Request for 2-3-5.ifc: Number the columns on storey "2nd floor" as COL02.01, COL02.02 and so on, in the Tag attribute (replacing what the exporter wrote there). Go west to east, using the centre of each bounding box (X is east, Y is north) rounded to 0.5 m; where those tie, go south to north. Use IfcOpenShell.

First a look at what the model holds.

```python
import ifcopenshell
import ifcopenshell.util.element
import ifcopenshell.util.placement

model = ifcopenshell.open("2-3-5.ifc")
print(model.schema)
storey = next(s for s in model.by_type("IfcBuildingStorey") if s.Name == "2nd floor")
columns = [e for e in ifcopenshell.util.element.get_decomposition(storey) if e.is_a("IfcColumn")]
for e in sorted(columns, key=lambda e: e.id()):
    origin = ifcopenshell.util.placement.get_local_placement(e.ObjectPlacement)[:3, 3]
    print(e.id(), e.Tag, e.Name, origin.round(2) + 0.0, sep=" | ")
```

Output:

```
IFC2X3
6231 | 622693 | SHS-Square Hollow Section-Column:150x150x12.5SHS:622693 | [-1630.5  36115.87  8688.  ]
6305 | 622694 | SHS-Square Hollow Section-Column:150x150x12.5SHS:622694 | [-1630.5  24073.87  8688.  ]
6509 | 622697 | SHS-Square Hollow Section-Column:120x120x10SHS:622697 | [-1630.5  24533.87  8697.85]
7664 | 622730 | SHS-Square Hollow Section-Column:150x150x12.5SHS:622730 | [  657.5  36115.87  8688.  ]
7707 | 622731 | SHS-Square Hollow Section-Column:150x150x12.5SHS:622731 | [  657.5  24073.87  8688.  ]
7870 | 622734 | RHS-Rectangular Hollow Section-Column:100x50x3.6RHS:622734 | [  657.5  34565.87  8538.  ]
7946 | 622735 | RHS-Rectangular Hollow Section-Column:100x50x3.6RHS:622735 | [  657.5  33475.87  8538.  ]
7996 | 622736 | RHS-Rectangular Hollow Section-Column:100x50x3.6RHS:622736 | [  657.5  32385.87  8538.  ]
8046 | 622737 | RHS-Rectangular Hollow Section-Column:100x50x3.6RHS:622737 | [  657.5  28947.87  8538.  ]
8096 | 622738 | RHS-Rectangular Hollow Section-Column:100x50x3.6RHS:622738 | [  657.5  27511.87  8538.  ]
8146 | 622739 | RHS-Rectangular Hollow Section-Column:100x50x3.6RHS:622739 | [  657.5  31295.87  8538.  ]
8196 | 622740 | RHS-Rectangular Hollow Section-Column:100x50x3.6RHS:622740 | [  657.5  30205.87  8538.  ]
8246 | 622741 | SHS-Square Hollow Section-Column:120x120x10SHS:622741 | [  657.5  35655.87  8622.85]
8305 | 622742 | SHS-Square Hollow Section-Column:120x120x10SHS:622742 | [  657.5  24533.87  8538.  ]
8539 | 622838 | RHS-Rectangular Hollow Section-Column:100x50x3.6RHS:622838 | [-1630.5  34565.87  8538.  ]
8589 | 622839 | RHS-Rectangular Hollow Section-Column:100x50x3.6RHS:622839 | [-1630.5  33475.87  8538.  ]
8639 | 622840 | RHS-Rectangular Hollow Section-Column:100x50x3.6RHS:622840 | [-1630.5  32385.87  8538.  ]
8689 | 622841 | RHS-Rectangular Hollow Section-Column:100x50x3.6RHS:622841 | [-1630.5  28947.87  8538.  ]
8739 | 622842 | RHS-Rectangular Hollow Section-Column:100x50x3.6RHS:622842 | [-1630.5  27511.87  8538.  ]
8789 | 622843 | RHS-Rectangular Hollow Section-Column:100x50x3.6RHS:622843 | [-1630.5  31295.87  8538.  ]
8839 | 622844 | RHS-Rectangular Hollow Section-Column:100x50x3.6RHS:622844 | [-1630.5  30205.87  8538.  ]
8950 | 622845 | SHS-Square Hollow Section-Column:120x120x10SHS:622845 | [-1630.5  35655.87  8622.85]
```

```python
import ifcopenshell
import ifcopenshell.geom
import ifcopenshell.util.element
import ifcopenshell.util.shape

model = ifcopenshell.open("2-3-5.ifc")
settings = ifcopenshell.geom.settings()
settings.set("use-world-coords", True)


def centre(element):
    shape = ifcopenshell.geom.create_shape(settings, element)
    return ifcopenshell.util.shape.get_bbox_centroid(shape.geometry)


storey = next(s for s in model.by_type("IfcBuildingStorey") if s.Name == "2nd floor")
columns = [e for e in ifcopenshell.util.element.get_decomposition(storey) if e.is_a("IfcColumn")]

# Insertion points can sit at a corner or the storey origin, so sort by the geometry (in metres).
centres = {e: centre(e) for e in columns}
columns.sort(key=lambda e: (round(centres[e][0] / 0.5), centres[e][1]))

for i, e in enumerate(columns, start=1):
    number = f"COL02.{i:02d}"
    e.Tag = number
    print(e.id(), number)

model.write("2-3-5_rev.ifc")
```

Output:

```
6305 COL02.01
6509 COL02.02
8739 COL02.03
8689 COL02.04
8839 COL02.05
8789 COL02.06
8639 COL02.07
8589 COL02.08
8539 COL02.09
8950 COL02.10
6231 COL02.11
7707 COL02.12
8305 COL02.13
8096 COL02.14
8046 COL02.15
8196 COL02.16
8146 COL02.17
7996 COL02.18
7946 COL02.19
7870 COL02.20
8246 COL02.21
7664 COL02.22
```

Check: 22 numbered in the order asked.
